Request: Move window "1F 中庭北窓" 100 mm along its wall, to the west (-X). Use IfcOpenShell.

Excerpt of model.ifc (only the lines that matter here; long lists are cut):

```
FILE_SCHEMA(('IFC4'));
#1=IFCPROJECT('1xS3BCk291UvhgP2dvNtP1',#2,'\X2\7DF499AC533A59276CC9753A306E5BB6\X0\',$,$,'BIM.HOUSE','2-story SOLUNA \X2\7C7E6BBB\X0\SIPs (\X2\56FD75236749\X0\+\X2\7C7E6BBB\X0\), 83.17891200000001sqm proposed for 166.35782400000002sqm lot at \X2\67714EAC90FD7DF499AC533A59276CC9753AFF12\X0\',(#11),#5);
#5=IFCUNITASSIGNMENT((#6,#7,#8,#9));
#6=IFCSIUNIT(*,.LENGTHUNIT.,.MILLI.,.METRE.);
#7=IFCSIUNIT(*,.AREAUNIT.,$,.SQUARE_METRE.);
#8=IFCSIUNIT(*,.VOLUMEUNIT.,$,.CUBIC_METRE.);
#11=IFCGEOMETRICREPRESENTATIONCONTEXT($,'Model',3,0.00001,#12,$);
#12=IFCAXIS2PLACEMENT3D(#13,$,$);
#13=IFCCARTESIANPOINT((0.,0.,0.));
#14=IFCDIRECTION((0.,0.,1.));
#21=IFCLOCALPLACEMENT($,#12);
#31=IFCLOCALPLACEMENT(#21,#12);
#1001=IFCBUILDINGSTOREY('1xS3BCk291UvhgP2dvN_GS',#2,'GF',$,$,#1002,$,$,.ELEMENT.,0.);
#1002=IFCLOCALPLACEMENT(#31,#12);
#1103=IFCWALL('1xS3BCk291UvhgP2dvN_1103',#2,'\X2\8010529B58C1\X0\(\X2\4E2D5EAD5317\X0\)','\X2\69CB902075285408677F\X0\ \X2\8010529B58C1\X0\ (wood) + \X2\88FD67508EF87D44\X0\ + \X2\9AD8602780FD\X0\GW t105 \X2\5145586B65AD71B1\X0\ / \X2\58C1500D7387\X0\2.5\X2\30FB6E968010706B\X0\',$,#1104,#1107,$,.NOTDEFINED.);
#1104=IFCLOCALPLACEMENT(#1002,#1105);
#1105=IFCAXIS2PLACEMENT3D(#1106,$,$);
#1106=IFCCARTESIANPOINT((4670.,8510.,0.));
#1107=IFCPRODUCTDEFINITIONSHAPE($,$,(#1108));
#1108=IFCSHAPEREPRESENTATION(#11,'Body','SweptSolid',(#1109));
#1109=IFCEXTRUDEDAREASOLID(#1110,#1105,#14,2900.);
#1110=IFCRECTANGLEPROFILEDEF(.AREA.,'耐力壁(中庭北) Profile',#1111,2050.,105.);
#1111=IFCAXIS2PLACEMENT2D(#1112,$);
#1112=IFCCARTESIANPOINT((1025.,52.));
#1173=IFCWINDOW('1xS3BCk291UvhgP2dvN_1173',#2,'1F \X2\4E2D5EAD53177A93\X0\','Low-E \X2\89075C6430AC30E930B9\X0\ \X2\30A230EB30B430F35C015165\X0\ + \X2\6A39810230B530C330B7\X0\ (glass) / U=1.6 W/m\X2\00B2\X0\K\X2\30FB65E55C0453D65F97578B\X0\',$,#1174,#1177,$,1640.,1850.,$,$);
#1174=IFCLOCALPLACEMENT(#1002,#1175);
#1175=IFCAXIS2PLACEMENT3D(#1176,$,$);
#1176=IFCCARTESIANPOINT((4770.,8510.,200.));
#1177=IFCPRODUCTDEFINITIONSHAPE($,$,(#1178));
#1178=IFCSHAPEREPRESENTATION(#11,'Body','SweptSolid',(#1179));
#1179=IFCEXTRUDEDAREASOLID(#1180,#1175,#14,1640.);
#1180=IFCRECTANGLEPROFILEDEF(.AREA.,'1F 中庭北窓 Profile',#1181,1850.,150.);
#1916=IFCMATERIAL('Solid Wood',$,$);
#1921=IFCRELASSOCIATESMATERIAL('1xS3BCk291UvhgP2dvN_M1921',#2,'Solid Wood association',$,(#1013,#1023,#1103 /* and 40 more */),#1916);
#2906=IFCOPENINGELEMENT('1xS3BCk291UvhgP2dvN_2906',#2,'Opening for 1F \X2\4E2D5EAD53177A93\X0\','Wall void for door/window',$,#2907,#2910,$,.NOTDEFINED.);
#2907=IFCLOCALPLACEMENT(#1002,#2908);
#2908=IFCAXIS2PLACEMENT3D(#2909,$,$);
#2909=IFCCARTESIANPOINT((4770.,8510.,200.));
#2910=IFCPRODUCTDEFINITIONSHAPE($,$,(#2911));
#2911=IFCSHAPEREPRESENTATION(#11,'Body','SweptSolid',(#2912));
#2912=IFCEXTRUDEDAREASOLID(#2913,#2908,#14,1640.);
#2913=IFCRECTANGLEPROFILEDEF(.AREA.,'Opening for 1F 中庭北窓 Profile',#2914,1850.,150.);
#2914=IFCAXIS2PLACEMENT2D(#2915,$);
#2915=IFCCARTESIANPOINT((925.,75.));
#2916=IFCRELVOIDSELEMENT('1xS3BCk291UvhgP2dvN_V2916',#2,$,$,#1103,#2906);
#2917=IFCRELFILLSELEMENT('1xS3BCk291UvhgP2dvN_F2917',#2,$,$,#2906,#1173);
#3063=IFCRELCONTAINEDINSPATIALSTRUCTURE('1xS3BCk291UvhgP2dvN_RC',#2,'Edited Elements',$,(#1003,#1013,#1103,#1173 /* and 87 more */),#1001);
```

```python
import ifcopenshell
import ifcopenshell.api.geometry
import ifcopenshell.util.placement
import ifcopenshell.util.unit

model = ifcopenshell.open("model.ifc")
unit_scale = ifcopenshell.util.unit.calculate_unit_scale(model)

window = model.by_guid("1xS3BCk291UvhgP2dvN_1173")
opening = window.FillsVoids[0].RelatingOpeningElement
wall = opening.VoidsElements[0].RelatingBuildingElement

wall_matrix = ifcopenshell.util.placement.get_local_placement(wall.ObjectPlacement)
shift = wall_matrix[:3, 0] * -0.1 / unit_scale
before = ifcopenshell.util.placement.get_local_placement(window.ObjectPlacement)[:3, 3].copy()

# The window is not placed relative to its opening, so move both.
for product in (opening, window):
    matrix = ifcopenshell.util.placement.get_local_placement(product.ObjectPlacement)
    matrix[:3, 3] += shift
    ifcopenshell.api.geometry.edit_object_placement(model, product=product, matrix=matrix, is_si=False)

after = ifcopenshell.util.placement.get_local_placement(window.ObjectPlacement)[:3, 3]
print("window moved by", (after - before).round(3) + 0.0)

model.write("model-out.ifc")
```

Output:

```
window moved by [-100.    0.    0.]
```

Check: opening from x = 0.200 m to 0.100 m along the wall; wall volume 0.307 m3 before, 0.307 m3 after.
